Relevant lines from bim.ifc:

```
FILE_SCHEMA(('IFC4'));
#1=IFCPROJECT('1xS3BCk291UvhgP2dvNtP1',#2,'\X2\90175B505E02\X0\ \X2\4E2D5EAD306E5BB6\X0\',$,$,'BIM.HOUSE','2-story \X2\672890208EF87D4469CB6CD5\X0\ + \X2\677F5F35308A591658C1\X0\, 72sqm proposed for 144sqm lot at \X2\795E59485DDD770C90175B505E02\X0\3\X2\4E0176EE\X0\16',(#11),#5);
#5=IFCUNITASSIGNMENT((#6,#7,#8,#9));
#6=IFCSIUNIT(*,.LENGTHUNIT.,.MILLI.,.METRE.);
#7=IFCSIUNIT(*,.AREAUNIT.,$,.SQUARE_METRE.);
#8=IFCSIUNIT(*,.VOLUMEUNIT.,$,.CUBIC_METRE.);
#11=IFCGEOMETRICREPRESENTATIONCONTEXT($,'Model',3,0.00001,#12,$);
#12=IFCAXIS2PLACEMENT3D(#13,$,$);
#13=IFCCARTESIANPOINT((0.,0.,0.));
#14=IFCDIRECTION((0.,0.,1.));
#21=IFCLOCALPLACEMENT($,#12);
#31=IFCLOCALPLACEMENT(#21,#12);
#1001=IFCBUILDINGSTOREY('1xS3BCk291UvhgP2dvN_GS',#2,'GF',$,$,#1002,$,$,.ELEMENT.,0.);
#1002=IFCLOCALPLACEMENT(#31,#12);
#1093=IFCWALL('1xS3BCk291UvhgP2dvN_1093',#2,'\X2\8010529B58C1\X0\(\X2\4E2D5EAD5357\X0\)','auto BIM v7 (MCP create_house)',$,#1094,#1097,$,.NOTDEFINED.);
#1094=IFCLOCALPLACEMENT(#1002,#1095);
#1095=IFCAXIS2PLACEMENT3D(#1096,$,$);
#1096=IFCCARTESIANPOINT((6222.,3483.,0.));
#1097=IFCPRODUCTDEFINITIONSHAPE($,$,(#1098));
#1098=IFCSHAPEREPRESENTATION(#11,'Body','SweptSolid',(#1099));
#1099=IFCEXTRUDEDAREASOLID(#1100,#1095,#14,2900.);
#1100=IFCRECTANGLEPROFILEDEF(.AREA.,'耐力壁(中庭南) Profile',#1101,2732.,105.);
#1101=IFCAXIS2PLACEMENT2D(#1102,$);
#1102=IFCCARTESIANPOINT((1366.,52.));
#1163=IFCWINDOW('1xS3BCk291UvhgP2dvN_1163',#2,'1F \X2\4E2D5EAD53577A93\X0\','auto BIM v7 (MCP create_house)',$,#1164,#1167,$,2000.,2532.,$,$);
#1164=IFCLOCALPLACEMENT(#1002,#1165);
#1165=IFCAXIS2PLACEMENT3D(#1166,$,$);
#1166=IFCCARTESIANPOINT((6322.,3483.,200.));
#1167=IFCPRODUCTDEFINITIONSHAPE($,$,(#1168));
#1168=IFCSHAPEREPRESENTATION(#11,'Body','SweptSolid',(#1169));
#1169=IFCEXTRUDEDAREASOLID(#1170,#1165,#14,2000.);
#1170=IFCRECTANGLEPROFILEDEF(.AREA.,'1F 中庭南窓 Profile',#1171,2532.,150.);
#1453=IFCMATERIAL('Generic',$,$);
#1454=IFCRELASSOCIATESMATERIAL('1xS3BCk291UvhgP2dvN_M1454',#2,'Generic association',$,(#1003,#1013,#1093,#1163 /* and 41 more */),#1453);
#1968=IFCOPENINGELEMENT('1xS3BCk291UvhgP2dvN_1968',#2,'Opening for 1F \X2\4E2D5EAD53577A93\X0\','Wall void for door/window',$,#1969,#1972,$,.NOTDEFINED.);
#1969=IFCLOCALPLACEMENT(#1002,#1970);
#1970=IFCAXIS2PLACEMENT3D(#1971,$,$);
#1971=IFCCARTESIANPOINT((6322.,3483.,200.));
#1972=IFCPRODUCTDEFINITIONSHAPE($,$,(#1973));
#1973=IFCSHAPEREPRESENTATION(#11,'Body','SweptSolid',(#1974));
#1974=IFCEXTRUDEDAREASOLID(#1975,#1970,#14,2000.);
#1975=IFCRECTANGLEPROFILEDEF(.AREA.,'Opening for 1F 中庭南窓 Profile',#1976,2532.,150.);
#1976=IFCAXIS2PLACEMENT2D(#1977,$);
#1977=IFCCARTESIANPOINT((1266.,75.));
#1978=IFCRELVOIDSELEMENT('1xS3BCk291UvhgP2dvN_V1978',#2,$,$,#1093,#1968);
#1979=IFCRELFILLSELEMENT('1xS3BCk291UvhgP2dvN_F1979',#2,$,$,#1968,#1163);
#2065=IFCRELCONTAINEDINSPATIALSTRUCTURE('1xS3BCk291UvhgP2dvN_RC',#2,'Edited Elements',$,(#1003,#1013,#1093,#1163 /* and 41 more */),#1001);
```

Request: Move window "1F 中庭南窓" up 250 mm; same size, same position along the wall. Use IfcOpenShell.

```python
import numpy as np
import ifcopenshell
import ifcopenshell.api.geometry
import ifcopenshell.util.placement
import ifcopenshell.util.unit

model = ifcopenshell.open("bim.ifc")
unit_scale = ifcopenshell.util.unit.calculate_unit_scale(model)

window = model.by_id(1163)
opening = window.FillsVoids[0].RelatingOpeningElement
dz = 0.25 / unit_scale

shift = np.array([0.0, 0.0, dz])
# The window is not placed relative to its opening, so move both.
for product in (opening, window):
    matrix = ifcopenshell.util.placement.get_local_placement(product.ObjectPlacement)
    matrix[:3, 3] += shift
    ifcopenshell.api.geometry.edit_object_placement(model, product=product, matrix=matrix, is_si=False)

print(f"moved by {dz * unit_scale:+.3f} m")

model.write("bim_edited.ifc")
```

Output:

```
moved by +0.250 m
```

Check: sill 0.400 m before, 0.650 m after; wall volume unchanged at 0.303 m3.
